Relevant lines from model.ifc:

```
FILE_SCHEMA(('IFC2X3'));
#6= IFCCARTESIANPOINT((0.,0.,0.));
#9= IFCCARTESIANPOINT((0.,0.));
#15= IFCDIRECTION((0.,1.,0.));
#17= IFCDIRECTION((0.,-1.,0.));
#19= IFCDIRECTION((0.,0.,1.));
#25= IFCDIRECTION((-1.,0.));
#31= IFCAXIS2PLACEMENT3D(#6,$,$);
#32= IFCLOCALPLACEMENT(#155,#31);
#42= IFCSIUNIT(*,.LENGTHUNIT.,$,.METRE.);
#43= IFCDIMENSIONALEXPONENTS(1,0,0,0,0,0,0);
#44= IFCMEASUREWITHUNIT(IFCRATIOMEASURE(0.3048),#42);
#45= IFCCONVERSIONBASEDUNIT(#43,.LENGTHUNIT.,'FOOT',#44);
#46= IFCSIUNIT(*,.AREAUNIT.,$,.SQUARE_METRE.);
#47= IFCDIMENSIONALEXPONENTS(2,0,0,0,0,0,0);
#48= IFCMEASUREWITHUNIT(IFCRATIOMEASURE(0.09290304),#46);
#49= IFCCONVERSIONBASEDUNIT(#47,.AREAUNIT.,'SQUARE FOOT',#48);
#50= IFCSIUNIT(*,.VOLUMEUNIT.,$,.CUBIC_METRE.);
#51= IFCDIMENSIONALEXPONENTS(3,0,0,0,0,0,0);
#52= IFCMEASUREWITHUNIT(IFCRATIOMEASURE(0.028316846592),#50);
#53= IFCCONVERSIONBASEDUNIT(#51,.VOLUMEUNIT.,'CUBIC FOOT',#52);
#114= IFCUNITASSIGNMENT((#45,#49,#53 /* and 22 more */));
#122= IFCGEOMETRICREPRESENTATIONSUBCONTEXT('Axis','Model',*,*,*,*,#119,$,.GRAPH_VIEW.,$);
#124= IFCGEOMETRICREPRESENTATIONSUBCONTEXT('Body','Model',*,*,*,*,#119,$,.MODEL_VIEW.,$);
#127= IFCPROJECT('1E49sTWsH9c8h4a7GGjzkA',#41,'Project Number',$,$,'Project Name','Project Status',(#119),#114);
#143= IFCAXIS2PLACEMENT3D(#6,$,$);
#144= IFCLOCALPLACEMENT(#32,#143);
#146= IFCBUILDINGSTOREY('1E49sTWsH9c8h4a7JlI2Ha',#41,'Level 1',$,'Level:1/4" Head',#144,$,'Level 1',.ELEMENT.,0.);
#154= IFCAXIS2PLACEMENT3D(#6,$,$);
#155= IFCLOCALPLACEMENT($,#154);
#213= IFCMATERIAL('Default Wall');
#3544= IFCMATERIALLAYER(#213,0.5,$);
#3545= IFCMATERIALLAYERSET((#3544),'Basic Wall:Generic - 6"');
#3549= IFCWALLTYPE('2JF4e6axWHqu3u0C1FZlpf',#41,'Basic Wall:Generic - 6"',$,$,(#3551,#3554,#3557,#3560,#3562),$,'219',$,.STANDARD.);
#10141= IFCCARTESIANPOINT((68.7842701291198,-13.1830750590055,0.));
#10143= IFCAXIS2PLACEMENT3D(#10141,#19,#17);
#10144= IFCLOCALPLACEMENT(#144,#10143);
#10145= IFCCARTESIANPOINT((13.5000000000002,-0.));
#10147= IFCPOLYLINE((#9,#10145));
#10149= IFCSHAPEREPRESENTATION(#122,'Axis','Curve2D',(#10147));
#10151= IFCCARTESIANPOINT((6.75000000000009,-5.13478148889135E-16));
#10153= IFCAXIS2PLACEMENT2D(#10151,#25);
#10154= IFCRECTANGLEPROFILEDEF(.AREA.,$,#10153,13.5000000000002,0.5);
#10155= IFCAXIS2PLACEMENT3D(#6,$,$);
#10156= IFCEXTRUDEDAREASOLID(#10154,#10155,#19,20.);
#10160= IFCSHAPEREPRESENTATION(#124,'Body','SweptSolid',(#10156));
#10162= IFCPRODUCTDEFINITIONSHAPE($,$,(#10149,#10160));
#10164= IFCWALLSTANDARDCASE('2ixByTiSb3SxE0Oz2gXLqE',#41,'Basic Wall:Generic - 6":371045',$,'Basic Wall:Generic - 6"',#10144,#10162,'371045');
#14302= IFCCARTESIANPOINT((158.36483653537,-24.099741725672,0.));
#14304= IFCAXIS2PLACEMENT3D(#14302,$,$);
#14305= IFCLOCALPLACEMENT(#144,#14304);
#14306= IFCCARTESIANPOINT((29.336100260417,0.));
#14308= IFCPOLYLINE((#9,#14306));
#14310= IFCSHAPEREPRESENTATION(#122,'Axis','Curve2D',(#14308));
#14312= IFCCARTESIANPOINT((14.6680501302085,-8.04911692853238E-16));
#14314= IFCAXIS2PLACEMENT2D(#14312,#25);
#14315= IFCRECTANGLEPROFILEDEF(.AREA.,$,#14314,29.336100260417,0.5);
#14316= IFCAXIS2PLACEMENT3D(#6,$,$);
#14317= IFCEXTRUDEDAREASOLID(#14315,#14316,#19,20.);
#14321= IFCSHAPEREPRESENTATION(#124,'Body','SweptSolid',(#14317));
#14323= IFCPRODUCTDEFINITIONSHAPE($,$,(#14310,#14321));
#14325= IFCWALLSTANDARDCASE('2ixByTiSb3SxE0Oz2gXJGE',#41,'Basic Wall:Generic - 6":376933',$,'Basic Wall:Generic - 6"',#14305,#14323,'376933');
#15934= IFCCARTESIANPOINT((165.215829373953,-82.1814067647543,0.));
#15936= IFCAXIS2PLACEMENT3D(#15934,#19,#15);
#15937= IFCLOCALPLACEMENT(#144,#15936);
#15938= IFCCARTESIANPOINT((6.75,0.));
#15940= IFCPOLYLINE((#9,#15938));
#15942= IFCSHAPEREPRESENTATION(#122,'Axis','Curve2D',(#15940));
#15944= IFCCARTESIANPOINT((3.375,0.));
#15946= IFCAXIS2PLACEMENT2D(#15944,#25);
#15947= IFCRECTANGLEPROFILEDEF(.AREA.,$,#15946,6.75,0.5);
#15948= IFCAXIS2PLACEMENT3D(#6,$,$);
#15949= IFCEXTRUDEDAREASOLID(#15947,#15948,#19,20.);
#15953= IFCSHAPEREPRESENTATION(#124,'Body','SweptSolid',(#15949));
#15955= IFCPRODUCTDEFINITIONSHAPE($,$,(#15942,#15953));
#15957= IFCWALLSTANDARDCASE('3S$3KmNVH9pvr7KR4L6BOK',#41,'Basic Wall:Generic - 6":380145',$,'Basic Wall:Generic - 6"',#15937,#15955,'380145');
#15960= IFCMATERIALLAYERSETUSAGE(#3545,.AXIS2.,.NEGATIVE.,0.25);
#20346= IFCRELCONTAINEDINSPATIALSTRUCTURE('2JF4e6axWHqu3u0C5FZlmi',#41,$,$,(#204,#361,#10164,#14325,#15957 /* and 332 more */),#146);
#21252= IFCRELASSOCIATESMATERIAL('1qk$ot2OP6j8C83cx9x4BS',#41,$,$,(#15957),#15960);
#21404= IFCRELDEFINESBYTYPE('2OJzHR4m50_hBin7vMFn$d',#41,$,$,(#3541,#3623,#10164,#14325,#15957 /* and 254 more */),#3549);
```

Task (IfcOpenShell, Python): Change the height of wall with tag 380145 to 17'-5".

```python
import ifcopenshell
import ifcopenshell.geom
import ifcopenshell.util.representation
import ifcopenshell.util.shape
import ifcopenshell.util.unit

model = ifcopenshell.open("model.ifc")
unit_scale = ifcopenshell.util.unit.calculate_unit_scale(model)
settings = ifcopenshell.geom.settings()


def volume(element):
    """Net volume in cubic metres, openings subtracted."""
    shape = ifcopenshell.geom.create_shape(settings, element)
    return ifcopenshell.util.shape.get_volume(shape.geometry)


wall = model.by_id(15957)
before = volume(wall)

body = ifcopenshell.util.representation.get_representation(wall, "Model", "Body")
solid = body.Items[0]
old_height = solid.Depth
solid.Depth = 209 * 0.0254 / unit_scale
after = volume(wall)

print(f"height {old_height:g} -> {solid.Depth:g}, volume {before:.3f} -> {after:.3f} m3")

model.write("model_rev.ifc")
```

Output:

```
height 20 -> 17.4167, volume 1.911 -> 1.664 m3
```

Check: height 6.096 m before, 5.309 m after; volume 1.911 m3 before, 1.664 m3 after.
